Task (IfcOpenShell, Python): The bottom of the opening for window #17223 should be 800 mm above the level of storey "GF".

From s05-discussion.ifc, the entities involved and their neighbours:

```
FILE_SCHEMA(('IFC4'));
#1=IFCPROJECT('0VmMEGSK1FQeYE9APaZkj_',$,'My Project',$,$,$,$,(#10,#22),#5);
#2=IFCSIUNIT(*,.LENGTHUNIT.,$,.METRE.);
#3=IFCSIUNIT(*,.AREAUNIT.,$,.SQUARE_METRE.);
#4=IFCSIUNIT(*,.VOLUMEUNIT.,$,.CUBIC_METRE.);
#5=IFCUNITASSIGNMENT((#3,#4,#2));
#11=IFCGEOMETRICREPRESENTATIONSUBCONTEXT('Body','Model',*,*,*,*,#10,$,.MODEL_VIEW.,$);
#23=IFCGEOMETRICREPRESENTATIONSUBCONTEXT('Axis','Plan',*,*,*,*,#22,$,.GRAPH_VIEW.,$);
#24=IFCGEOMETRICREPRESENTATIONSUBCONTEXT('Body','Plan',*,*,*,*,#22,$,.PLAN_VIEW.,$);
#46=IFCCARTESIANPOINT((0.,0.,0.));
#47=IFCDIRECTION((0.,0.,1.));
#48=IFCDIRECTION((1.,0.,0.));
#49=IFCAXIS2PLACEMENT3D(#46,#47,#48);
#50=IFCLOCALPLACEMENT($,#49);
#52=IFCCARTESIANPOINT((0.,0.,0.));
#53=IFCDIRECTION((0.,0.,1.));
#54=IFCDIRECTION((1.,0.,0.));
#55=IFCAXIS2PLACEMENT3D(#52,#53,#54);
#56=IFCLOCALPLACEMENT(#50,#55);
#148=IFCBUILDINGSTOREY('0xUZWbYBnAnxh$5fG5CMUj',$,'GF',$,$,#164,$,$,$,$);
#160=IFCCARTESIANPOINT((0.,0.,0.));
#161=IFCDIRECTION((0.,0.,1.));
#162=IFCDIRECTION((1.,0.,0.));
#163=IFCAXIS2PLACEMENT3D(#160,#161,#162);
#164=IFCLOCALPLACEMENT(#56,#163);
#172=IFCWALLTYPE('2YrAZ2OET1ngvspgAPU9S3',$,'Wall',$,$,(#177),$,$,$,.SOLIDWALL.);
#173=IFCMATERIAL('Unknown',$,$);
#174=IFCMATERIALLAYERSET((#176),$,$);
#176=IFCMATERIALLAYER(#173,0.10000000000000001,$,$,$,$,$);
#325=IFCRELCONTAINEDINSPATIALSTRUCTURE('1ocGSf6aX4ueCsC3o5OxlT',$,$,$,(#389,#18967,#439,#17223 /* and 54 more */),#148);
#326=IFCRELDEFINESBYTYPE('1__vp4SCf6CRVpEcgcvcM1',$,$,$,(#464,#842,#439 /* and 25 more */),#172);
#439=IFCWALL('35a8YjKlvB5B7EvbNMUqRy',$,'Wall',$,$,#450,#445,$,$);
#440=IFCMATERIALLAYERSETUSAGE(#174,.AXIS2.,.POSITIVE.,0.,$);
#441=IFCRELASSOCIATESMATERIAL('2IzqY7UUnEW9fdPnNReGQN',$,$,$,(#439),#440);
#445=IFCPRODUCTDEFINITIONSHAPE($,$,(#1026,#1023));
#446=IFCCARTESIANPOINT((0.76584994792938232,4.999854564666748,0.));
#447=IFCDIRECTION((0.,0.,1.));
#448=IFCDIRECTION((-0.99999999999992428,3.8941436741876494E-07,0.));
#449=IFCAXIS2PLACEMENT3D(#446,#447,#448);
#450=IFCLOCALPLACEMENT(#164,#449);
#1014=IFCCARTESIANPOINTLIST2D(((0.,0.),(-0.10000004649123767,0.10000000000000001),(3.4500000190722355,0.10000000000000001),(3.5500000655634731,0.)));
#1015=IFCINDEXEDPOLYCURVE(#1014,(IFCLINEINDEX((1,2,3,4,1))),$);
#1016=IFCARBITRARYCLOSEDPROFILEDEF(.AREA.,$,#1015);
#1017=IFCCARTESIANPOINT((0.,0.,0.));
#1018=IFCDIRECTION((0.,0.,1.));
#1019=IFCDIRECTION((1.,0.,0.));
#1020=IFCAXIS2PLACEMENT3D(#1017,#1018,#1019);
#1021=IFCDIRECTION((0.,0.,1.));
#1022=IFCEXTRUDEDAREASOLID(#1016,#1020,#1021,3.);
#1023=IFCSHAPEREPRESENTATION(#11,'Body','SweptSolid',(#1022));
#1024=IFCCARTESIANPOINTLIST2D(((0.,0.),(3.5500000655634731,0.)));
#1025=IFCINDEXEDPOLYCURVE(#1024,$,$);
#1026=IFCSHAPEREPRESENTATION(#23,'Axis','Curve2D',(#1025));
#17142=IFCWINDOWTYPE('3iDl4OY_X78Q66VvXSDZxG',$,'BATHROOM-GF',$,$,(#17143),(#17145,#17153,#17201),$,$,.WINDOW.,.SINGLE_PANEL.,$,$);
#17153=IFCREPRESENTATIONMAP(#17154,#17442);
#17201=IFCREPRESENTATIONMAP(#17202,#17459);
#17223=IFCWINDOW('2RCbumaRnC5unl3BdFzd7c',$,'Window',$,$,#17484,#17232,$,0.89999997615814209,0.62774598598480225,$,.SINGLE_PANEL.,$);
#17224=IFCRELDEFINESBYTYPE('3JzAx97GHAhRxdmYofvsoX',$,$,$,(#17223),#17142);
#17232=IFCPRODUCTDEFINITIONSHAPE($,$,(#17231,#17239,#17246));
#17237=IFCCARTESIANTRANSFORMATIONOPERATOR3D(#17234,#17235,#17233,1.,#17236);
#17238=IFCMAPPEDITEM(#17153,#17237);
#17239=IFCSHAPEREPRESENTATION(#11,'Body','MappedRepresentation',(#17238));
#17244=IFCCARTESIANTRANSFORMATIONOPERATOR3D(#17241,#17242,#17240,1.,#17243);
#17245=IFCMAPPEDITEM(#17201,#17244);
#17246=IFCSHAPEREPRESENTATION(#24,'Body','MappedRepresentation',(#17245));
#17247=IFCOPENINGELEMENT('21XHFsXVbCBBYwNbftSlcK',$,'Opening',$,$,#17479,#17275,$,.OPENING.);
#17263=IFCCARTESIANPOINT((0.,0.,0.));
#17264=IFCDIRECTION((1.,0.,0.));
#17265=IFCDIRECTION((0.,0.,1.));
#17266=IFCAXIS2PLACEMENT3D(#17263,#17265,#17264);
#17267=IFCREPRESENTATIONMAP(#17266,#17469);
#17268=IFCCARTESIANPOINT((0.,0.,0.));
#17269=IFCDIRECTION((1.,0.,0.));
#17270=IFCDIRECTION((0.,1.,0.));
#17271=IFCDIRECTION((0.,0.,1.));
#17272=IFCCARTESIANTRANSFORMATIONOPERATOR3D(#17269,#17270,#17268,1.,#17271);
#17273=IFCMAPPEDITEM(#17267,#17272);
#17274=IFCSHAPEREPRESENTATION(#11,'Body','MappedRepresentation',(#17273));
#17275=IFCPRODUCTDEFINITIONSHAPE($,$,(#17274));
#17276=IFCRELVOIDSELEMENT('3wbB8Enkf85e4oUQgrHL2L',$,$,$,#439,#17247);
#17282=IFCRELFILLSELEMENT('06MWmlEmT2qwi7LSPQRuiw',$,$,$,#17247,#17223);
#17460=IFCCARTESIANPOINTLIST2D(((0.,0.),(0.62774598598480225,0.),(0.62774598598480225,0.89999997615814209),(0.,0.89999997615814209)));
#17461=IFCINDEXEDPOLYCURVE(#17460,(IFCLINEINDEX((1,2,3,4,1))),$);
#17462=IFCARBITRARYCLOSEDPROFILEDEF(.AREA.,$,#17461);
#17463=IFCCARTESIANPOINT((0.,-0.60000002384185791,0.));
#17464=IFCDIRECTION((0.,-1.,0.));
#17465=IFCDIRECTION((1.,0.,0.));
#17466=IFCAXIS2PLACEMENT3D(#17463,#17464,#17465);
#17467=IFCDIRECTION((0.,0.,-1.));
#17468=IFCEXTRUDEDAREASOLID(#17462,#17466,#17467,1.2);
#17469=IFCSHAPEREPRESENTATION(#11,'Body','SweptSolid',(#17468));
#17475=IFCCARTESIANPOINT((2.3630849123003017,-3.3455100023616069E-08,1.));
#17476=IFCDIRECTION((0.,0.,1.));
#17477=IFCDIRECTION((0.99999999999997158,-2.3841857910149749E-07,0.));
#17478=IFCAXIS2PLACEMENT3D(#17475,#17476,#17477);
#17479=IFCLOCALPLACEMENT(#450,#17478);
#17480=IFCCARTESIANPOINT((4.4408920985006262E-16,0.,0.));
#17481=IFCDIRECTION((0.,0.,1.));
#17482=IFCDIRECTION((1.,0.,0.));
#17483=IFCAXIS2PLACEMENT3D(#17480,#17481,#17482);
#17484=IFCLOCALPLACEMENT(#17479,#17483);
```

```python
import numpy as np
import ifcopenshell
import ifcopenshell.api.geometry
import ifcopenshell.geom
import ifcopenshell.util.element
import ifcopenshell.util.placement
import ifcopenshell.util.shape
import ifcopenshell.util.unit

model = ifcopenshell.open("s05-discussion.ifc")
unit_scale = ifcopenshell.util.unit.calculate_unit_scale(model)

window = model.by_id(17223)
opening = window.FillsVoids[0].RelatingOpeningElement
storey = ifcopenshell.util.element.get_container(window, ifc_class="IfcBuildingStorey")
level = ifcopenshell.util.placement.get_local_placement(storey.ObjectPlacement)[2, 3]

# The opening's origin need not be at the sill, so measure its lowest point.
shape = ifcopenshell.geom.create_shape(ifcopenshell.geom.settings(), opening)
bottom = ifcopenshell.util.shape.get_shape_bottom_elevation(shape, shape.geometry) / unit_scale
dz = level + 0.8 / unit_scale - bottom

shift = np.array([0.0, 0.0, dz])
# The window is placed relative to its opening, so it follows when the opening moves.
matrix = ifcopenshell.util.placement.get_local_placement(opening.ObjectPlacement)
matrix[:3, 3] += shift
ifcopenshell.api.geometry.edit_object_placement(
    model, product=opening, matrix=matrix, is_si=False, should_transform_children=True
)

print(f"moved by {dz * unit_scale:+.3f} m")

model.write("s05-discussion_updated.ifc")
```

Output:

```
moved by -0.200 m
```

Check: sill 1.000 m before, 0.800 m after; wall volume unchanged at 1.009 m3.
